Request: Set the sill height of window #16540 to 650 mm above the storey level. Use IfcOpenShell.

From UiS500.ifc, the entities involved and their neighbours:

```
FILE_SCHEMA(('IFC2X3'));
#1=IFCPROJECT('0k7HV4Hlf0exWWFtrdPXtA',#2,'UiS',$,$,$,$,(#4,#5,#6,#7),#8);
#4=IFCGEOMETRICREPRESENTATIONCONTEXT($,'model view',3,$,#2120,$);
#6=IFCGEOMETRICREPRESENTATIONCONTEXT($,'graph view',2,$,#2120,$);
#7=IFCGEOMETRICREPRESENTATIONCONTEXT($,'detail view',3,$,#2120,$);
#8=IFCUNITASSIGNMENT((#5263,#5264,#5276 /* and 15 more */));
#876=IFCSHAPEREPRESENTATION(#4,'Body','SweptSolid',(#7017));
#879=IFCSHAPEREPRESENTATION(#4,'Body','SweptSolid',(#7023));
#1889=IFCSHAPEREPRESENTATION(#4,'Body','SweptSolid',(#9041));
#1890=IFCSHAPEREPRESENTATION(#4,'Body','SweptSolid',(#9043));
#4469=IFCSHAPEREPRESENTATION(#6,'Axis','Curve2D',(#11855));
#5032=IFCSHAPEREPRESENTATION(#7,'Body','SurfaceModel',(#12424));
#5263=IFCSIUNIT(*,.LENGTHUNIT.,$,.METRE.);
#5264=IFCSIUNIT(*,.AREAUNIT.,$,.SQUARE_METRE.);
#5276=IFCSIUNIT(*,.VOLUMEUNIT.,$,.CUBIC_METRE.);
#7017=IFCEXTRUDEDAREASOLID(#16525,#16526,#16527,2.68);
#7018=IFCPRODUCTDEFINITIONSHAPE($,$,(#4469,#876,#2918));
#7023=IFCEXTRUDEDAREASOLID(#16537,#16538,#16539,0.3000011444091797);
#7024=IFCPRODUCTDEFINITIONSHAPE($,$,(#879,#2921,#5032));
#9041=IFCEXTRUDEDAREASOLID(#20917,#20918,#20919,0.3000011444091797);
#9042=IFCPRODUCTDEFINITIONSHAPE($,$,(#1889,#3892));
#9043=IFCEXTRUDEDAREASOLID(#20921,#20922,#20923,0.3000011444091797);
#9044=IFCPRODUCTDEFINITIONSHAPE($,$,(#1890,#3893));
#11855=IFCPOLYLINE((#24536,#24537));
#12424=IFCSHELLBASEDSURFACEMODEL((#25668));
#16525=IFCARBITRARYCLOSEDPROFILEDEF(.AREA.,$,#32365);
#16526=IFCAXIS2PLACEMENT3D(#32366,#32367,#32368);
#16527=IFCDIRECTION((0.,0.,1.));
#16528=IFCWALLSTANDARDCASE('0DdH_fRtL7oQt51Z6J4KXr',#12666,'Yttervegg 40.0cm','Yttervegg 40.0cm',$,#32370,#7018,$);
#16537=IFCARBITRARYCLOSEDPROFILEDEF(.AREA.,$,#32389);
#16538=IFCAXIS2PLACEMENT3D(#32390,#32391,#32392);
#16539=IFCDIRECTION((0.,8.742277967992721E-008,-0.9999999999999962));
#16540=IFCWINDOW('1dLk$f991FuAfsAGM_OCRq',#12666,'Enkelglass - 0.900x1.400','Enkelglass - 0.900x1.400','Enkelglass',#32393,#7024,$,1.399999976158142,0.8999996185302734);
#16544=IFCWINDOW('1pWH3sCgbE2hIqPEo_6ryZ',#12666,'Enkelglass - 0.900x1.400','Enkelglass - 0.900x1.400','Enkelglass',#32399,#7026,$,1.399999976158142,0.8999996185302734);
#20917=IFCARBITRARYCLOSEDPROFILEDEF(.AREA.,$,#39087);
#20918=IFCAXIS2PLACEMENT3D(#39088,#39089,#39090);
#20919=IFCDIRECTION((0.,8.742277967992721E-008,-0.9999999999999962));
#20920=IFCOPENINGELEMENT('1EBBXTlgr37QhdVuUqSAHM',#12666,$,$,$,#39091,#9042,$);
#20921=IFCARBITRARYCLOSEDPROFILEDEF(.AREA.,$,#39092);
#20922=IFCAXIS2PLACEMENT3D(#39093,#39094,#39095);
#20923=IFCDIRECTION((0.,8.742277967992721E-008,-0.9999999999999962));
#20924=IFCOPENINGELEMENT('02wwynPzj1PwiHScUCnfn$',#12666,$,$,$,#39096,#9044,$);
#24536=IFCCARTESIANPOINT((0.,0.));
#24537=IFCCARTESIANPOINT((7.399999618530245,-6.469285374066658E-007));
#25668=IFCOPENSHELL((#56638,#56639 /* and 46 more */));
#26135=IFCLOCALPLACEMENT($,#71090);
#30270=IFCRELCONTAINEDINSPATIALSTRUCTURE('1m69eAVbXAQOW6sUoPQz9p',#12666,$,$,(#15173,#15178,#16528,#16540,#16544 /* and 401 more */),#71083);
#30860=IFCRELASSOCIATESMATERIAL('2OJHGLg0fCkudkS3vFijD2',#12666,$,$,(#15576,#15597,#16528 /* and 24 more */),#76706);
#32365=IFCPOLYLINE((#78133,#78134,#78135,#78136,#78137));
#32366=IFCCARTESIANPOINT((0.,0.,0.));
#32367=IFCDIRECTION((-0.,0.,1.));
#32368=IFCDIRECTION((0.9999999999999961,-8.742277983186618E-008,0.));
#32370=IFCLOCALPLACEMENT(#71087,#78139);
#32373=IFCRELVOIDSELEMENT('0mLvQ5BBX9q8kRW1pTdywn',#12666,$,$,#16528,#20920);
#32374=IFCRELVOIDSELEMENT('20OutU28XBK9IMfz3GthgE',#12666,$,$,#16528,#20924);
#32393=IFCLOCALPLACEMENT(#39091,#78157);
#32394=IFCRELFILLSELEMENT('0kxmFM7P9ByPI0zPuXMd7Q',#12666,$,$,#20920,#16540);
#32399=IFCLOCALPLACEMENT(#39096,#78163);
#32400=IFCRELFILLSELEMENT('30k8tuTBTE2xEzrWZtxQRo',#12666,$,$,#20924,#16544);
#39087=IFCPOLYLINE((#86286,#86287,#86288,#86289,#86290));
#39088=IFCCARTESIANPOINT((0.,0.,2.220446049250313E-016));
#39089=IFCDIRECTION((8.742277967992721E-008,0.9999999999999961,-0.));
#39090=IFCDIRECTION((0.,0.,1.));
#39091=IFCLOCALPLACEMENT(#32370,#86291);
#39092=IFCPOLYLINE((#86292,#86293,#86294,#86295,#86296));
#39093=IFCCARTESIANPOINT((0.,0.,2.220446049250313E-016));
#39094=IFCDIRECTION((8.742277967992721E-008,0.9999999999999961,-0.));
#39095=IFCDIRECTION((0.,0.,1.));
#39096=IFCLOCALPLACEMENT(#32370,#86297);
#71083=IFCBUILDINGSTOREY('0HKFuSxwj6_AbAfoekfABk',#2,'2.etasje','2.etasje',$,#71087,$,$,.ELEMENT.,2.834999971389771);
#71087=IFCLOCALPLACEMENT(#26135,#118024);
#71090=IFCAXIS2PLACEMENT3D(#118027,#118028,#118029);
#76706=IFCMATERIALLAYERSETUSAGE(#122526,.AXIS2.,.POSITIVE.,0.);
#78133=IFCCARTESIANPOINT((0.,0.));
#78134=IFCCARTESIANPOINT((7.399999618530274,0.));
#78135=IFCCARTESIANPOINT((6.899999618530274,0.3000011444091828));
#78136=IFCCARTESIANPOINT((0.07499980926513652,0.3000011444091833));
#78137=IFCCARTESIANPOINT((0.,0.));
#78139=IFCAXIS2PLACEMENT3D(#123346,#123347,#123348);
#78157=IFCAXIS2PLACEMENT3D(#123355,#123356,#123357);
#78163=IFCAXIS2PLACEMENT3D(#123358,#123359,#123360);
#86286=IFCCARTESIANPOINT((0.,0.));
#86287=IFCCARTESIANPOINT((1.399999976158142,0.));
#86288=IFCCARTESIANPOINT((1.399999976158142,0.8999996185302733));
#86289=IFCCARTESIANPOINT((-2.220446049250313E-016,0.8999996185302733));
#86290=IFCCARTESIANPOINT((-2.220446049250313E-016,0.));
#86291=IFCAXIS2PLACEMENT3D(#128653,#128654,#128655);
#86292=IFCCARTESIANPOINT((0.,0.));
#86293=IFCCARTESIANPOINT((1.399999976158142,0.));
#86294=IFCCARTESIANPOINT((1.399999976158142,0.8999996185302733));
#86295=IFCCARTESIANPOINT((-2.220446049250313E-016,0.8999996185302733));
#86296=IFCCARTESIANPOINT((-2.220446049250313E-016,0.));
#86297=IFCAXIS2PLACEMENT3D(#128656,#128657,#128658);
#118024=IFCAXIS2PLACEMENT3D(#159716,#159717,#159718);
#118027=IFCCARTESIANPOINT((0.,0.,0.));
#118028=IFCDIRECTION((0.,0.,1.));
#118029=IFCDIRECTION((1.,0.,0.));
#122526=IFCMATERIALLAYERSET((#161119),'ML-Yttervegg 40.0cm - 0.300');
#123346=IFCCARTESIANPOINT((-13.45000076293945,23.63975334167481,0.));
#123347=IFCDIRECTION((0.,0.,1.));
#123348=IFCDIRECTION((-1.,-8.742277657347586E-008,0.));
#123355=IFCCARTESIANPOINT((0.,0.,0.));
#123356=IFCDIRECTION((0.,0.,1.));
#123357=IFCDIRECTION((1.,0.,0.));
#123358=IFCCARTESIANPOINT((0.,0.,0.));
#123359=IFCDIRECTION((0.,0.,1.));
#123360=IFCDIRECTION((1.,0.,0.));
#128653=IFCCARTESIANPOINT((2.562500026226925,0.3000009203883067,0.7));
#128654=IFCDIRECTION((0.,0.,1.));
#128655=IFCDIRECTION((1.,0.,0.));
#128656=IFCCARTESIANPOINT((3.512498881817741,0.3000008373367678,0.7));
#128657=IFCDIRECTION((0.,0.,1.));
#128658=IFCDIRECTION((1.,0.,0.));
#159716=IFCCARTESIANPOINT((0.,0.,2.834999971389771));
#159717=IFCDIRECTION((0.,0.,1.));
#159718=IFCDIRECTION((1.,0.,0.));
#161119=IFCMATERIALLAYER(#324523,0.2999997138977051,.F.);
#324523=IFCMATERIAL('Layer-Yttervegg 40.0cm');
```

```python
import numpy as np
import ifcopenshell
import ifcopenshell.api.geometry
import ifcopenshell.geom
import ifcopenshell.util.element
import ifcopenshell.util.placement
import ifcopenshell.util.shape
import ifcopenshell.util.unit

model = ifcopenshell.open("UiS500.ifc")
unit_scale = ifcopenshell.util.unit.calculate_unit_scale(model)

window = model.by_guid("1dLk$f991FuAfsAGM_OCRq")
opening = window.FillsVoids[0].RelatingOpeningElement
storey = ifcopenshell.util.element.get_container(window, ifc_class="IfcBuildingStorey")
level = ifcopenshell.util.placement.get_local_placement(storey.ObjectPlacement)[2, 3]

# The opening's origin need not be at the sill, so measure its lowest point.
shape = ifcopenshell.geom.create_shape(ifcopenshell.geom.settings(), opening)
bottom = ifcopenshell.util.shape.get_shape_bottom_elevation(shape, shape.geometry) / unit_scale
dz = level + 0.65 / unit_scale - bottom

shift = np.array([0.0, 0.0, dz])
# The window is placed relative to its opening, so it follows when the opening moves.
matrix = ifcopenshell.util.placement.get_local_placement(opening.ObjectPlacement)
matrix[:3, 3] += shift
ifcopenshell.api.geometry.edit_object_placement(
    model, product=opening, matrix=matrix, is_si=False, should_transform_children=True
)

print(f"moved by {dz * unit_scale:+.3f} m")

model.write("UiS500_rev.ifc")
```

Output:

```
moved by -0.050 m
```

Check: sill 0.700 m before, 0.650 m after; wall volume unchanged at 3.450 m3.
